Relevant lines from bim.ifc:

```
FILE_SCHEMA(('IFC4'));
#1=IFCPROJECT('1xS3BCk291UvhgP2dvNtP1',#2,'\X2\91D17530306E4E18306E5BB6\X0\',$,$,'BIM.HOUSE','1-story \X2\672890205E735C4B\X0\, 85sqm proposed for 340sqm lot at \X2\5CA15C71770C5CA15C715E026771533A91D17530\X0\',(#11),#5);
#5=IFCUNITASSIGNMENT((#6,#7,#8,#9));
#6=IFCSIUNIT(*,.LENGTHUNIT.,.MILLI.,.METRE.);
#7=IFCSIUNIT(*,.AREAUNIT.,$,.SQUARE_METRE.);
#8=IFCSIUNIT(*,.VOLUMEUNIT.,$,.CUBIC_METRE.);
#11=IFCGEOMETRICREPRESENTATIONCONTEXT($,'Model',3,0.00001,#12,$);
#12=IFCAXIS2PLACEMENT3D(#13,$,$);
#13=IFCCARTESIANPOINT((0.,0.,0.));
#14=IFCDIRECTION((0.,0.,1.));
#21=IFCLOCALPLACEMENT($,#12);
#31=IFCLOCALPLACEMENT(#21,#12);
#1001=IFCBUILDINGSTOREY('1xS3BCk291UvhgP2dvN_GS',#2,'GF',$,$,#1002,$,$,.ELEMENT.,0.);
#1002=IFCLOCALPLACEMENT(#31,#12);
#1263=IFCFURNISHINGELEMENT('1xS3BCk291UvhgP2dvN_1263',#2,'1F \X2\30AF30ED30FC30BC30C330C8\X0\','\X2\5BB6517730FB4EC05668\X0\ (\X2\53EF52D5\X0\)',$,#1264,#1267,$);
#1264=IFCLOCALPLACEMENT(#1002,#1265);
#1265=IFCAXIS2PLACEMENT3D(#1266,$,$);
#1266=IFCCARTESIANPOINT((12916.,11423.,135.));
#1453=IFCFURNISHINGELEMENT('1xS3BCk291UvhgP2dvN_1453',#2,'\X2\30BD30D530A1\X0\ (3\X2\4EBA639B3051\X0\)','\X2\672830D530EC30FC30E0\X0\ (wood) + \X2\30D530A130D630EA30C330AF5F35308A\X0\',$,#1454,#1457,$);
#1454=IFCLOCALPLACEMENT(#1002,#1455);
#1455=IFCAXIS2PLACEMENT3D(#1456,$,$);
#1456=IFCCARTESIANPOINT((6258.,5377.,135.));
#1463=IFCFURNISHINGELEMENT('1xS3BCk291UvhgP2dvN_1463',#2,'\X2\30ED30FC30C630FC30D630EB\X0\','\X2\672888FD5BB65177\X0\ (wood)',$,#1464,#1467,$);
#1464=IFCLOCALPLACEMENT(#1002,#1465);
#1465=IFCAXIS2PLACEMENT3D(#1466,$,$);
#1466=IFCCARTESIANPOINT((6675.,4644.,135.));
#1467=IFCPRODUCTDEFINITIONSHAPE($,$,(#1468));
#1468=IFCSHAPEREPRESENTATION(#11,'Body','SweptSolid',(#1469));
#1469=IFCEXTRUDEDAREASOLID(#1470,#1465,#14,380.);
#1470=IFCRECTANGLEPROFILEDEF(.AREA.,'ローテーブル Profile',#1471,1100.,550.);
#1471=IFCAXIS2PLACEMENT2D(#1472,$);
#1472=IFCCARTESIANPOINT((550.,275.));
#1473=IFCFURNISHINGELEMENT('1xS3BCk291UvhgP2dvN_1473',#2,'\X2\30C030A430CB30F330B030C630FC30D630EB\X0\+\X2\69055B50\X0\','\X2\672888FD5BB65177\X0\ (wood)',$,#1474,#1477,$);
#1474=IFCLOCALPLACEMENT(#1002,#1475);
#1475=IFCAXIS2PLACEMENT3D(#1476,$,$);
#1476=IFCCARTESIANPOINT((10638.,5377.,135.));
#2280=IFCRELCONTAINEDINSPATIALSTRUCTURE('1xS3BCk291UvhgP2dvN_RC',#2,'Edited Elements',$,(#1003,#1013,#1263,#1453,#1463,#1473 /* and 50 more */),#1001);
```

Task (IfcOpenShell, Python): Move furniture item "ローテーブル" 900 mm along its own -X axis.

```python
import ifcopenshell
import ifcopenshell.api.geometry
import ifcopenshell.util.placement
import ifcopenshell.util.unit

model = ifcopenshell.open("bim.ifc")
unit_scale = ifcopenshell.util.unit.calculate_unit_scale(model)

item = model.by_guid("1xS3BCk291UvhgP2dvN_1463")
matrix = ifcopenshell.util.placement.get_local_placement(item.ObjectPlacement)
matrix[:3, 3] -= matrix[:3, 0] * 0.9 / unit_scale
ifcopenshell.api.geometry.edit_object_placement(model, product=item, matrix=matrix, is_si=False)

print(ifcopenshell.util.placement.get_local_placement(item.ObjectPlacement).round(3) + 0.0)

model.write("bim_updated.ifc")
```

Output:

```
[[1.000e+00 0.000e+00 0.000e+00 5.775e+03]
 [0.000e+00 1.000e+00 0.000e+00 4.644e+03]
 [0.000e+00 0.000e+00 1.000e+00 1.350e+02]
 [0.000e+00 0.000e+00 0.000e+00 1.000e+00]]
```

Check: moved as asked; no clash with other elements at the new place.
